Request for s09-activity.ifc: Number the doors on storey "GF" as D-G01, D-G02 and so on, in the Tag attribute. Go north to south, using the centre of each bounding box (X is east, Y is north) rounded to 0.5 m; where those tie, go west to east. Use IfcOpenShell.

First a look at what the model holds.

```python
import ifcopenshell
import ifcopenshell.util.element
import ifcopenshell.util.placement

model = ifcopenshell.open("s09-activity.ifc")
print(model.schema)
storey = next(s for s in model.by_type("IfcBuildingStorey") if s.Name == "GF")
doors = [e for e in ifcopenshell.util.element.get_decomposition(storey) if e.is_a("IfcDoor")]
for e in sorted(doors, key=lambda e: e.id()):
    origin = ifcopenshell.util.placement.get_local_placement(e.ObjectPlacement)[:3, 3]
    print(e.id(), e.Tag, e.Name, origin.round(2) + 0.0, sep=" | ")
```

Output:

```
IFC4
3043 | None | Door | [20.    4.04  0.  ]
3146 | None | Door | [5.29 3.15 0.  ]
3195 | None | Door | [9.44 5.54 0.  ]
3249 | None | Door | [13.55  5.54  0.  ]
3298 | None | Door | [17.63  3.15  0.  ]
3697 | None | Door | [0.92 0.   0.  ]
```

```python
import ifcopenshell
import ifcopenshell.geom
import ifcopenshell.util.element
import ifcopenshell.util.shape

model = ifcopenshell.open("s09-activity.ifc")
settings = ifcopenshell.geom.settings()
settings.set("use-world-coords", True)


def centre(element):
    shape = ifcopenshell.geom.create_shape(settings, element)
    return ifcopenshell.util.shape.get_bbox_centroid(shape.geometry)


storey = next(s for s in model.by_type("IfcBuildingStorey") if s.Name == "GF")
doors = [e for e in ifcopenshell.util.element.get_decomposition(storey) if e.is_a("IfcDoor")]

# Insertion points can sit at a corner or the storey origin, so sort by the geometry (in metres).
centres = {e: centre(e) for e in doors}
doors.sort(key=lambda e: (-round(centres[e][1] / 0.5), centres[e][0]))

for i, e in enumerate(doors, start=1):
    number = f"D-G{i:02d}"
    e.Tag = number
    print(e.id(), number)

model.write("s09-activity_edited.ifc")
```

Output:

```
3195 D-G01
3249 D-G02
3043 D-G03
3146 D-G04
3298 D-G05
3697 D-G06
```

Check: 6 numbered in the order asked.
